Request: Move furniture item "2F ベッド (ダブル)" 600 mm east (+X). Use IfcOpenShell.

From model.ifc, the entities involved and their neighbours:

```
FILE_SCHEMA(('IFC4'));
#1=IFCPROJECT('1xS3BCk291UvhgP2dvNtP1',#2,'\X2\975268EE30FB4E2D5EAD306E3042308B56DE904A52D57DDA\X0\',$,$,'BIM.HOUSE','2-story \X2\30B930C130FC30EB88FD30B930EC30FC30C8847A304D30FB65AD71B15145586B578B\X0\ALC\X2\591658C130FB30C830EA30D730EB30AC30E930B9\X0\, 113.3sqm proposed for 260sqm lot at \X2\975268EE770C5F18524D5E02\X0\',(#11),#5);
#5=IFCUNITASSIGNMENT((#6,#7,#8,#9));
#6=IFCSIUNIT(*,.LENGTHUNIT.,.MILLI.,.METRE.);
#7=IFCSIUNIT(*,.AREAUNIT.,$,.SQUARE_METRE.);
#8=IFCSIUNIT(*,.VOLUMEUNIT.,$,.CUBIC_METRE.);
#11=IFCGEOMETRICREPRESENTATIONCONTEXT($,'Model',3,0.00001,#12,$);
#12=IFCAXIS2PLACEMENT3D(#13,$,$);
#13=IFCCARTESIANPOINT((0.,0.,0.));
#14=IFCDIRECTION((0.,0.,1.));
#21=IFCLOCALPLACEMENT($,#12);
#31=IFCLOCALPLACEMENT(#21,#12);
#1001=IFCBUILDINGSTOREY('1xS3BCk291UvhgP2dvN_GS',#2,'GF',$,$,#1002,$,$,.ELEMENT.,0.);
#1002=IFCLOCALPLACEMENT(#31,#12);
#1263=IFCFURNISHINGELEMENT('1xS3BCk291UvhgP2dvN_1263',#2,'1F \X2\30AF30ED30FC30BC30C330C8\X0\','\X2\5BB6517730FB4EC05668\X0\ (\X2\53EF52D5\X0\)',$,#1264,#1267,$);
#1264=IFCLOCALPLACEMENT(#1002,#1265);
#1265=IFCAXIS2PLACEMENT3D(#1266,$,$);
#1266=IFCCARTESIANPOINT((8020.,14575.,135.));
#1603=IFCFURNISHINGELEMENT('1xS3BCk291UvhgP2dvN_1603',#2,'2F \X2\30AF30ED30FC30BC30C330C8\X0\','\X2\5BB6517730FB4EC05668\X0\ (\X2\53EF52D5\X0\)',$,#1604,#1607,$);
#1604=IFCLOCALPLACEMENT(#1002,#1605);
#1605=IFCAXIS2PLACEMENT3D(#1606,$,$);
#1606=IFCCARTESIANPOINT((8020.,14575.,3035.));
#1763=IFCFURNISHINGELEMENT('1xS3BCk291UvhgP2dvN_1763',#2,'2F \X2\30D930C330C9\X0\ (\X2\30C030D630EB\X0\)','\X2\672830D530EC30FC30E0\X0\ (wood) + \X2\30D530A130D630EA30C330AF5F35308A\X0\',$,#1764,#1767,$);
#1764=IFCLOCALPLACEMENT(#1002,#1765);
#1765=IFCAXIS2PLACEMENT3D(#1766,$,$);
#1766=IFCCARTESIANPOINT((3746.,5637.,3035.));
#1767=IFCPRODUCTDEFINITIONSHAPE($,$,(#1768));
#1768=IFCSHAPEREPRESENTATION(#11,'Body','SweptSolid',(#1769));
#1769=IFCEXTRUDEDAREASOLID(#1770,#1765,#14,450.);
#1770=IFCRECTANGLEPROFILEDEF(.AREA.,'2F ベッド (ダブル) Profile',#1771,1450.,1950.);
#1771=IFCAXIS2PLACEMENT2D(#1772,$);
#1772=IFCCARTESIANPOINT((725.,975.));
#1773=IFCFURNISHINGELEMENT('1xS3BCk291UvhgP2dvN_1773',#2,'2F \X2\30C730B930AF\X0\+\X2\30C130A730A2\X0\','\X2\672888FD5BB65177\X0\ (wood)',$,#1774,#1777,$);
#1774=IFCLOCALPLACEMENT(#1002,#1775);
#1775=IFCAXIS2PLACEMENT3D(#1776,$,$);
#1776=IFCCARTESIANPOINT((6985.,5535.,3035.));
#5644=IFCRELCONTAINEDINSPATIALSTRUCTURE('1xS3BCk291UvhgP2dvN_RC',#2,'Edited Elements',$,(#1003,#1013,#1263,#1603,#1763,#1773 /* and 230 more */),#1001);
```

```python
import ifcopenshell
import ifcopenshell.api.geometry
import ifcopenshell.util.placement
import ifcopenshell.util.unit

model = ifcopenshell.open("model.ifc")
unit_scale = ifcopenshell.util.unit.calculate_unit_scale(model)

item = model.by_guid("1xS3BCk291UvhgP2dvN_1763")
matrix = ifcopenshell.util.placement.get_local_placement(item.ObjectPlacement)
matrix[0, 3] += 0.6 / unit_scale
ifcopenshell.api.geometry.edit_object_placement(model, product=item, matrix=matrix, is_si=False)

print(ifcopenshell.util.placement.get_local_placement(item.ObjectPlacement).round(3) + 0.0)

model.write("model_edited.ifc")
```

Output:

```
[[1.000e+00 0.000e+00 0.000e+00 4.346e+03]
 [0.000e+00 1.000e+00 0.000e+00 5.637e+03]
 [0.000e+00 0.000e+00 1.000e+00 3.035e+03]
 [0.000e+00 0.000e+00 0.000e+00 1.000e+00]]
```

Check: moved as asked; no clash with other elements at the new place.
